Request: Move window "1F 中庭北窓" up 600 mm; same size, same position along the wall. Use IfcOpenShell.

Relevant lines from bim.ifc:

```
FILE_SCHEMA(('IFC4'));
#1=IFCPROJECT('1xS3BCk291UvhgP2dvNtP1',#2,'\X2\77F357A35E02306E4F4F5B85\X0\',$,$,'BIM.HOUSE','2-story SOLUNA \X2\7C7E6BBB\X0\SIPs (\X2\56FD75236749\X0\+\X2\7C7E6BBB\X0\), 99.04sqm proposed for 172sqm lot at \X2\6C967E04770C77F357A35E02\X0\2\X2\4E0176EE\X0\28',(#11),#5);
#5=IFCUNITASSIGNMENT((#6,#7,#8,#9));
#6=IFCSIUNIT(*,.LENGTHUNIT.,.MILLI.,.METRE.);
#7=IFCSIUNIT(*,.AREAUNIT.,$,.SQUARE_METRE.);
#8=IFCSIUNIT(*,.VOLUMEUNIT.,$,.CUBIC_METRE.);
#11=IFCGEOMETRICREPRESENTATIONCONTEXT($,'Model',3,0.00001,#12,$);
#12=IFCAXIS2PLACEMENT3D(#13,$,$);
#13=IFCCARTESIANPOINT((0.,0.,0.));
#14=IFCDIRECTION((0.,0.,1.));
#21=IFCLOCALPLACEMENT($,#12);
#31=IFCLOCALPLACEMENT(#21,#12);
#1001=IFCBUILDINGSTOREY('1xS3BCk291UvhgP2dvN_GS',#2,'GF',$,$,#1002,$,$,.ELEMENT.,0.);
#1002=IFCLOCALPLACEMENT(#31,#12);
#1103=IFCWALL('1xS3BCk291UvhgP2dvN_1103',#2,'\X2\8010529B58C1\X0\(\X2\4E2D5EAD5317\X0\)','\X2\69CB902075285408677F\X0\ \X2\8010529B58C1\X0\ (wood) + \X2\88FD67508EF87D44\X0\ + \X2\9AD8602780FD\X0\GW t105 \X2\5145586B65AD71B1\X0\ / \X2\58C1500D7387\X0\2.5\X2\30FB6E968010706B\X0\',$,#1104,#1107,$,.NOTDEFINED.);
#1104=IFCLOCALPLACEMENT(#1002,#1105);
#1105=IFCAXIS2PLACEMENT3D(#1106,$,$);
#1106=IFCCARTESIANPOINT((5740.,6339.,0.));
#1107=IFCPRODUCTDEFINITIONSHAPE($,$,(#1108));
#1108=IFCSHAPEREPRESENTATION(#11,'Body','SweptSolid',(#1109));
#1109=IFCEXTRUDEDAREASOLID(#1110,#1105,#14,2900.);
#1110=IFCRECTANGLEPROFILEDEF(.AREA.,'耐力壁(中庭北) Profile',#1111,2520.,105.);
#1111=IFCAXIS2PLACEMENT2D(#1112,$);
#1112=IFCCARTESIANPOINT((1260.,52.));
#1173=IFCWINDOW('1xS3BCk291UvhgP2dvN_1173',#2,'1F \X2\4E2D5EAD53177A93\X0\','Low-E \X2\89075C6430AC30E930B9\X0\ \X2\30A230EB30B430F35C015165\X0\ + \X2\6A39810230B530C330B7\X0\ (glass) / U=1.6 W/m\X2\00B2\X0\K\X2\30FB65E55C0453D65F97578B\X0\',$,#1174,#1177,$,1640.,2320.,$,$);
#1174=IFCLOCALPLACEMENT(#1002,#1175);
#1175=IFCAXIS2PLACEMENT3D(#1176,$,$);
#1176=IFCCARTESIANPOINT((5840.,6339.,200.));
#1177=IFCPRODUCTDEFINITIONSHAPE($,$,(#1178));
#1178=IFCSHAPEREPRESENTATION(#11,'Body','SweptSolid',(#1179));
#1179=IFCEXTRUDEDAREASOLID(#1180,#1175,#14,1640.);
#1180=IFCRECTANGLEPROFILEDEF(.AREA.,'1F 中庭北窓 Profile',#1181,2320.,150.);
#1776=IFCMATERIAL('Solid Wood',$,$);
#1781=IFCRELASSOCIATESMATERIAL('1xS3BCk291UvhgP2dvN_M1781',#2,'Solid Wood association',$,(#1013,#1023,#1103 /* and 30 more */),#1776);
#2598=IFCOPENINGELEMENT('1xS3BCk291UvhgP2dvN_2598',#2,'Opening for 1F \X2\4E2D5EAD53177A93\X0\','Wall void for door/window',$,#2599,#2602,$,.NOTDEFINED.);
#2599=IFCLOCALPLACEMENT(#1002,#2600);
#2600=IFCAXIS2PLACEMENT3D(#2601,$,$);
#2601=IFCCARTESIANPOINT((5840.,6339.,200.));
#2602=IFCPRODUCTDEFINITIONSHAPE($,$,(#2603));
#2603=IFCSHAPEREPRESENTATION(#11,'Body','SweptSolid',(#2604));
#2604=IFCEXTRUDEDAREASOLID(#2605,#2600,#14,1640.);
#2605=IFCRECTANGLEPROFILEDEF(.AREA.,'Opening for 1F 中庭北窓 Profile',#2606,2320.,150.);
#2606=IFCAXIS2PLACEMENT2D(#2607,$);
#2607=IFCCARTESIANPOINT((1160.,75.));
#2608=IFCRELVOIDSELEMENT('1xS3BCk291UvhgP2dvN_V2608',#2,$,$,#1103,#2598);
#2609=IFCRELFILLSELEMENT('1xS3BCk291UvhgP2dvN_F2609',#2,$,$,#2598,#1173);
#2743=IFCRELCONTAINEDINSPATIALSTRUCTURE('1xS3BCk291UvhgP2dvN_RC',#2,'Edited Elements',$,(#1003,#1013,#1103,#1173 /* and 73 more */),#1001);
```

```python
import numpy as np
import ifcopenshell
import ifcopenshell.api.geometry
import ifcopenshell.util.placement
import ifcopenshell.util.unit

model = ifcopenshell.open("bim.ifc")
unit_scale = ifcopenshell.util.unit.calculate_unit_scale(model)

window = model.by_guid("1xS3BCk291UvhgP2dvN_1173")
opening = window.FillsVoids[0].RelatingOpeningElement
dz = 0.6 / unit_scale

shift = np.array([0.0, 0.0, dz])
# The window is not placed relative to its opening, so move both.
for product in (opening, window):
    matrix = ifcopenshell.util.placement.get_local_placement(product.ObjectPlacement)
    matrix[:3, 3] += shift
    ifcopenshell.api.geometry.edit_object_placement(model, product=product, matrix=matrix, is_si=False)

print(f"moved by {dz * unit_scale:+.3f} m")

model.write("bim_edited.ifc")
```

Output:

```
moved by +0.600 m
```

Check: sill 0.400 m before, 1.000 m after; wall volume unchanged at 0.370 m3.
